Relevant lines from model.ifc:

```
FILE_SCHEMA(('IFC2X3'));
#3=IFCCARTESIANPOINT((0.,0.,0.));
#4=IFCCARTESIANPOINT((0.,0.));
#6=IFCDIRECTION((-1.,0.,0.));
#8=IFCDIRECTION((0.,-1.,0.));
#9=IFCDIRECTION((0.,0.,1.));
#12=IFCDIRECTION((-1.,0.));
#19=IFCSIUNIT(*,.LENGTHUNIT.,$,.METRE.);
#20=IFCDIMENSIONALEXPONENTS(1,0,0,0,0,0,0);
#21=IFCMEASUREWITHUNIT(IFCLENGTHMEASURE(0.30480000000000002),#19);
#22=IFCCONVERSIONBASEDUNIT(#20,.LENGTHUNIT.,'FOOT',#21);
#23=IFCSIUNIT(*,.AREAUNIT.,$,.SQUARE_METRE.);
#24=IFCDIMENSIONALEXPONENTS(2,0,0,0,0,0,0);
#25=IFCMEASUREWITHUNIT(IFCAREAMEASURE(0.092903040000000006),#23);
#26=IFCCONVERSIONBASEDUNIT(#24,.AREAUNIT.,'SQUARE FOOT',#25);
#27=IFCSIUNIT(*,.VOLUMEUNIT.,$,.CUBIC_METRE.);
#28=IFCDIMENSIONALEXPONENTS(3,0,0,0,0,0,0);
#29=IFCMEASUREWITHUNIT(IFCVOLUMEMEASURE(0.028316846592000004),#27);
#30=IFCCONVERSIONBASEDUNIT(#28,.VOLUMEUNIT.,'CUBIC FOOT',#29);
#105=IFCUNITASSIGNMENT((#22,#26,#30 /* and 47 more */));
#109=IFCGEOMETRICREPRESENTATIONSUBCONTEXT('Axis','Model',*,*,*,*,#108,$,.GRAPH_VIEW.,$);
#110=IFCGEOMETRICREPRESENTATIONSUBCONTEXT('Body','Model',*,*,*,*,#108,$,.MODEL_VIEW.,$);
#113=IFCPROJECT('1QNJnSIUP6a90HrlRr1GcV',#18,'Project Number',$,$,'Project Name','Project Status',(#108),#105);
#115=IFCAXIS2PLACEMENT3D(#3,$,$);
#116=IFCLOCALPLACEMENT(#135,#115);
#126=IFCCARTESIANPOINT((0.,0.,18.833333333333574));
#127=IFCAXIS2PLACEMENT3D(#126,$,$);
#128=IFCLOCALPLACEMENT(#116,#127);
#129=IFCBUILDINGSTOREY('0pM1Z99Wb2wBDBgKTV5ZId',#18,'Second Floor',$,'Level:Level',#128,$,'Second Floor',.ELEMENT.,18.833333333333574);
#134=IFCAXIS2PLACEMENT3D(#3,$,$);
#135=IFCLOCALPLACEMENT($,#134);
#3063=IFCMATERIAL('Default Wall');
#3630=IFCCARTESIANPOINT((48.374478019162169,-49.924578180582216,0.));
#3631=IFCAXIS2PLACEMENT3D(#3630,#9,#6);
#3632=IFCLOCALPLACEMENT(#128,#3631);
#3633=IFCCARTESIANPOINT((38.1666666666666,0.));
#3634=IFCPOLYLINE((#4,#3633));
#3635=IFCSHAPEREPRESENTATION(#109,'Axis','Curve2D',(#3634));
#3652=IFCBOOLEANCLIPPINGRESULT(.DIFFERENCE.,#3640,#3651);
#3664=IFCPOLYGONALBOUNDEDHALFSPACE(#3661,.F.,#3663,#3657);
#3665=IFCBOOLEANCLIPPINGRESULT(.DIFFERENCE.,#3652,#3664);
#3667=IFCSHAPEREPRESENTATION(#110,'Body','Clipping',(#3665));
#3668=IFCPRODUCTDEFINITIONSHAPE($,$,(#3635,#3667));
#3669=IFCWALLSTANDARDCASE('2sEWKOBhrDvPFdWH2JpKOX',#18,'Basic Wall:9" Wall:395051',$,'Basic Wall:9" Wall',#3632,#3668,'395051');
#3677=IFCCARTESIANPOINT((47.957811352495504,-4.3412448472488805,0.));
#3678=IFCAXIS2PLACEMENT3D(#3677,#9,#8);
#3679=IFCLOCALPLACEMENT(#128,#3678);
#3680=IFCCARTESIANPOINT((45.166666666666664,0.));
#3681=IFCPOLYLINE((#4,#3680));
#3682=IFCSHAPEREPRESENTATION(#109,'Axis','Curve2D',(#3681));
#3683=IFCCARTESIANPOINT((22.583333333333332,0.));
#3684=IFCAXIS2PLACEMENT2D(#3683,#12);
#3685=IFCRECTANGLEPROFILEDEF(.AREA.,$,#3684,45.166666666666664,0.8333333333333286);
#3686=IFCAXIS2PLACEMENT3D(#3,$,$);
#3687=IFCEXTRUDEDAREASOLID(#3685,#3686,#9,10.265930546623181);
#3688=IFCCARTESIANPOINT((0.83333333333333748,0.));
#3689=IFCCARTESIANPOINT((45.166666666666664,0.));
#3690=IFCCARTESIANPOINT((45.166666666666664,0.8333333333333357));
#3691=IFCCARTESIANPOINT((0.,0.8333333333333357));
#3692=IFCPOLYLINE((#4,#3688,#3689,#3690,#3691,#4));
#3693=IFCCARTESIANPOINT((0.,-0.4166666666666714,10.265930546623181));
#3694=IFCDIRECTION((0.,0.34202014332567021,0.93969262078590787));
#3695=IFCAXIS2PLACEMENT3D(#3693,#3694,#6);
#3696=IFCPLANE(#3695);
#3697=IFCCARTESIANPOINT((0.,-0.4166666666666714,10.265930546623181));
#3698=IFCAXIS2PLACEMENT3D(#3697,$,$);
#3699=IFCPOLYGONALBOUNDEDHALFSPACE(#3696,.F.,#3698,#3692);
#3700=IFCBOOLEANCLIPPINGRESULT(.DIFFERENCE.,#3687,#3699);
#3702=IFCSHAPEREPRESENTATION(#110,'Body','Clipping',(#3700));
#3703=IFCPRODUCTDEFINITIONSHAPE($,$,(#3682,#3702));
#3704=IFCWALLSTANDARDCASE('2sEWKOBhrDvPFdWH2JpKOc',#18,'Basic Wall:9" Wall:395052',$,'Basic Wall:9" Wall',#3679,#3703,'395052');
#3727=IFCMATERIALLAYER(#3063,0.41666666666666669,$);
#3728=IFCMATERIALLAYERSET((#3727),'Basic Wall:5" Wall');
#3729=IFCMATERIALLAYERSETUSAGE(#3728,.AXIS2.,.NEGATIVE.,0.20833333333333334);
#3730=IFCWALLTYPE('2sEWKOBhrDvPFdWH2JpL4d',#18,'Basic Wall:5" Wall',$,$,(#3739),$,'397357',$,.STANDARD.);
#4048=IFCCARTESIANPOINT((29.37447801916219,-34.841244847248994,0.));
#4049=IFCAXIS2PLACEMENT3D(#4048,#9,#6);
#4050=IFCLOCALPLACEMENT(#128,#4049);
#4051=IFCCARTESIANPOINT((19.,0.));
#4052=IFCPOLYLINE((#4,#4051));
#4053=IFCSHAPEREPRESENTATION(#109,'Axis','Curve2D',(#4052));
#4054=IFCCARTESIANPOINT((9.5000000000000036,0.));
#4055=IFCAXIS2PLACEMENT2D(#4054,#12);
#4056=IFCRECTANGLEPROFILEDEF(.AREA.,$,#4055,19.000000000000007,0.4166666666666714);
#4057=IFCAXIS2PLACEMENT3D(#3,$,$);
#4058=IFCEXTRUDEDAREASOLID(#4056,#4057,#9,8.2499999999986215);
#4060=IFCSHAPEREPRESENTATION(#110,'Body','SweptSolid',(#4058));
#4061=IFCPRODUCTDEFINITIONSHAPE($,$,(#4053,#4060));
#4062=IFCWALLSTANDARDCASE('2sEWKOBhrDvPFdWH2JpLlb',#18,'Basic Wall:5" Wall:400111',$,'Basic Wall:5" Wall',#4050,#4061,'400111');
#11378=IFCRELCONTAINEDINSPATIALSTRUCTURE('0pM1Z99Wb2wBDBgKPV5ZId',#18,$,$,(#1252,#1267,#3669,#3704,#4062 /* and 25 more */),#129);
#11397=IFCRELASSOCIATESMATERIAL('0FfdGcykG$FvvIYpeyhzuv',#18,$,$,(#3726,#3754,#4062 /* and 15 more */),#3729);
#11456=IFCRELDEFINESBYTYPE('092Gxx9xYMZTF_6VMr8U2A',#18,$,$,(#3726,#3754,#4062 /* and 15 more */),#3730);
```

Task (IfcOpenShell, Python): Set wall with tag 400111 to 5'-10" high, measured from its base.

```python
import ifcopenshell
import ifcopenshell.geom
import ifcopenshell.util.representation
import ifcopenshell.util.shape
import ifcopenshell.util.unit

model = ifcopenshell.open("model.ifc")
unit_scale = ifcopenshell.util.unit.calculate_unit_scale(model)
settings = ifcopenshell.geom.settings()


def volume(element):
    """Net volume in cubic metres, openings subtracted."""
    shape = ifcopenshell.geom.create_shape(settings, element)
    return ifcopenshell.util.shape.get_volume(shape.geometry)


wall = model.by_guid("2sEWKOBhrDvPFdWH2JpLlb")
before = volume(wall)

body = ifcopenshell.util.representation.get_representation(wall, "Model", "Body")
solid = body.Items[0]
old_height = solid.Depth
solid.Depth = 70 * 0.0254 / unit_scale
after = volume(wall)

print(f"height {old_height:g} -> {solid.Depth:g}, volume {before:.3f} -> {after:.3f} m3")

model.write("model-out.ifc")
```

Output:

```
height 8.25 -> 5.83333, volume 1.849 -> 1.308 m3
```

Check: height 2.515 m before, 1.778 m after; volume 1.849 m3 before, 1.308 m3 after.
